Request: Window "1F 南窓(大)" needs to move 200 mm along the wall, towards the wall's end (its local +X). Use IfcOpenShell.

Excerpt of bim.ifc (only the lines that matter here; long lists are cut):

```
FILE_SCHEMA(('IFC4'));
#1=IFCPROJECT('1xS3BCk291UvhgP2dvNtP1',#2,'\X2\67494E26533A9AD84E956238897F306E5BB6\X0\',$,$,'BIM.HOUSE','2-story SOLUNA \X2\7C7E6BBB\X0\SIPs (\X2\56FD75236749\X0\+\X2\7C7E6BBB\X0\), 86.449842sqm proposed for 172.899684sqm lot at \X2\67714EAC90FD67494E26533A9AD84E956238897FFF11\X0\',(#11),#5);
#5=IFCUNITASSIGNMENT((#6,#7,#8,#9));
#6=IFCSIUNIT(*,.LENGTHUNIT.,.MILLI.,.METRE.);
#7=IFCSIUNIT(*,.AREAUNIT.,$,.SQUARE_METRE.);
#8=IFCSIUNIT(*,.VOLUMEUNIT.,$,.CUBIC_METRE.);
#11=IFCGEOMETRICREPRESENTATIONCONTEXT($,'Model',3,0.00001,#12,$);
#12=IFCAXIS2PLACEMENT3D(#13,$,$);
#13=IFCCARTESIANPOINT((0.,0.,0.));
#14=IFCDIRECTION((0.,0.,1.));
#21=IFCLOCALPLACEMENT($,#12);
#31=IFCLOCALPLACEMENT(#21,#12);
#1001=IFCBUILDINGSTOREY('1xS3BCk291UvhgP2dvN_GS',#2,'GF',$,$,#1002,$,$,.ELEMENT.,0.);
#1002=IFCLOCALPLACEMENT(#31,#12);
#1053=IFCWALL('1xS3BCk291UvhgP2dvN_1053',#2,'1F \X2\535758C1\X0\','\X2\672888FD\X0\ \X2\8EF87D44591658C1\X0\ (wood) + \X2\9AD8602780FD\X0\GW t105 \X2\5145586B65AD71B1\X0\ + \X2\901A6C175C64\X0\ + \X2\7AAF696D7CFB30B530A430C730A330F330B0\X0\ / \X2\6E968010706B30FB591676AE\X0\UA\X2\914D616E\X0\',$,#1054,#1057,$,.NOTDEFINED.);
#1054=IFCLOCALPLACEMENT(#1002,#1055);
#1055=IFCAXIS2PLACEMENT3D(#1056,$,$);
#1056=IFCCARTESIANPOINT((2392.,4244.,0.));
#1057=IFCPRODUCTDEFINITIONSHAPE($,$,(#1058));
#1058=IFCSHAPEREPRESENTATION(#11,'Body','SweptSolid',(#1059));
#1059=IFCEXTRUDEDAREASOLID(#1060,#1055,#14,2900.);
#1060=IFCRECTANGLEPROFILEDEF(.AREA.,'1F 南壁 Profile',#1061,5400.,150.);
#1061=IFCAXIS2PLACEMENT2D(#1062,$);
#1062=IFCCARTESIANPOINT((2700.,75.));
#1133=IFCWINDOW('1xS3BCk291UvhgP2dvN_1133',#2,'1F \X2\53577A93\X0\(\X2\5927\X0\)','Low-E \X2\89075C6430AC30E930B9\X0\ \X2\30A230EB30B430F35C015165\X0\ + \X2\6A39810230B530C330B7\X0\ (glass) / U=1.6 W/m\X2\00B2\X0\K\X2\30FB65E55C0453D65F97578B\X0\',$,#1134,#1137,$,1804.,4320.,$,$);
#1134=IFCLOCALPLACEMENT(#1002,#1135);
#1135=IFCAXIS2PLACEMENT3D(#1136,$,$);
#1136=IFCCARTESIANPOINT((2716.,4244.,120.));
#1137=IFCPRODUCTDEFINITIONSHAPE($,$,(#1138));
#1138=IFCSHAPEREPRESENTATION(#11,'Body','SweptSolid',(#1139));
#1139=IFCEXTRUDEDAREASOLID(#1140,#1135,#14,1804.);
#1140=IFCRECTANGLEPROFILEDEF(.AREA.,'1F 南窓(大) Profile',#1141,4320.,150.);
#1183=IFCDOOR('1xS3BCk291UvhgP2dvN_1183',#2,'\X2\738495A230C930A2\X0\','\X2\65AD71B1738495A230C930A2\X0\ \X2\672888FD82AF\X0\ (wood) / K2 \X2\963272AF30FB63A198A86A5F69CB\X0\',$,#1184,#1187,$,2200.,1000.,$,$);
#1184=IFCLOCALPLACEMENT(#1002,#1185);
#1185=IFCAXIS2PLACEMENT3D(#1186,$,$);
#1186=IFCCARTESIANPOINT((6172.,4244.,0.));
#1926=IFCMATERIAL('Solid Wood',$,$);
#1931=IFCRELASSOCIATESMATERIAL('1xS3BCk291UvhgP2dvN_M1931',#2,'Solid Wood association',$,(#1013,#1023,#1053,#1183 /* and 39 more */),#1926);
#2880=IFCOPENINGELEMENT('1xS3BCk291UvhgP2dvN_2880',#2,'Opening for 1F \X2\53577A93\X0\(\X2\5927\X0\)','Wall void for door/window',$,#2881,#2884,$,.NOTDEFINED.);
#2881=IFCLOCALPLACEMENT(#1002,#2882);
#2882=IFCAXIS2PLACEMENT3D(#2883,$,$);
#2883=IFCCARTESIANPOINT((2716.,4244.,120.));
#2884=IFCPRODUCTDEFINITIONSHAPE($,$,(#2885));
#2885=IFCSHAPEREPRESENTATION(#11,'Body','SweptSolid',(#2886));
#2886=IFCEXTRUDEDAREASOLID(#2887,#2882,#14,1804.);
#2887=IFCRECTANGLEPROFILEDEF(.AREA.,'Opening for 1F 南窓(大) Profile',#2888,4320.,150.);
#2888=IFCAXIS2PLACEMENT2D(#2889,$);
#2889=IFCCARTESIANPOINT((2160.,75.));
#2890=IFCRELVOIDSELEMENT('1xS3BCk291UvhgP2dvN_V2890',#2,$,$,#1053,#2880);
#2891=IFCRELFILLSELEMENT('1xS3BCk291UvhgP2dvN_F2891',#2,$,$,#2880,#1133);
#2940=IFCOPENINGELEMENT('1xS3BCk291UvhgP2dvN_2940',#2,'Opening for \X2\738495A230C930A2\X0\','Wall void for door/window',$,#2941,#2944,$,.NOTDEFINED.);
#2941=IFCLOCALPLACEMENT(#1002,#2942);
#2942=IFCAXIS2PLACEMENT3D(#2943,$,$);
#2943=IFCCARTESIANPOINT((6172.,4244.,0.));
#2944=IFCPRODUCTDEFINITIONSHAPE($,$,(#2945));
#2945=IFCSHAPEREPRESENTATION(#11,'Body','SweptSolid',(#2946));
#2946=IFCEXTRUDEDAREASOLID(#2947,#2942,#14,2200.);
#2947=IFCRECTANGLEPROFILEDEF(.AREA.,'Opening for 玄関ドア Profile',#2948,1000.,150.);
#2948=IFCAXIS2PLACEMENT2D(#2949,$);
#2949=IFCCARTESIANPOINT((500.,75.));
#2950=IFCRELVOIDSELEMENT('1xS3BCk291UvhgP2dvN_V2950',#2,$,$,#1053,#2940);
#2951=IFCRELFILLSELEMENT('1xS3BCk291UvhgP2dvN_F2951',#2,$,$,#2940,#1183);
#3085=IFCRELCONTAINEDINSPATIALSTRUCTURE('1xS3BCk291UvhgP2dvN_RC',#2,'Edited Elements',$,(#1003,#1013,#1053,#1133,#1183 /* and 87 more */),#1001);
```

```python
import ifcopenshell
import ifcopenshell.api.geometry
import ifcopenshell.util.placement
import ifcopenshell.util.unit

model = ifcopenshell.open("bim.ifc")
unit_scale = ifcopenshell.util.unit.calculate_unit_scale(model)

window = model.by_guid("1xS3BCk291UvhgP2dvN_1133")
opening = window.FillsVoids[0].RelatingOpeningElement
wall = opening.VoidsElements[0].RelatingBuildingElement

wall_matrix = ifcopenshell.util.placement.get_local_placement(wall.ObjectPlacement)
shift = wall_matrix[:3, 0] * 0.2 / unit_scale
before = ifcopenshell.util.placement.get_local_placement(window.ObjectPlacement)[:3, 3].copy()

# The window is not placed relative to its opening, so move both.
for product in (opening, window):
    matrix = ifcopenshell.util.placement.get_local_placement(product.ObjectPlacement)
    matrix[:3, 3] += shift
    ifcopenshell.api.geometry.edit_object_placement(model, product=product, matrix=matrix, is_si=False)

after = ifcopenshell.util.placement.get_local_placement(window.ObjectPlacement)[:3, 3]
print("window moved by", (after - before).round(3) + 0.0)

model.write("bim_updated.ifc")
```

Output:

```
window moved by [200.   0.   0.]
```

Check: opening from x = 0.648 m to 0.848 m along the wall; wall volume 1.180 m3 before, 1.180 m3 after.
